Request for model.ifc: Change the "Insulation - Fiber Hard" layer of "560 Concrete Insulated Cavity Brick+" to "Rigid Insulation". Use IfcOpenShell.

First a look at what the model holds.

```python
import ifcopenshell
import ifcopenshell.util.element

model = ifcopenshell.open("model.ifc")
print(model.schema)
for layer_set in model.by_type("IfcMaterialLayerSet"):
    if layer_set.LayerSetName == "560 Concrete Insulated Cavity Brick+":
        for layer in layer_set.MaterialLayers:
            print(layer.id(), layer.Material and layer.Material.Name, layer.LayerThickness, sep=" | ")
        print(len(ifcopenshell.util.element.get_elements_by_material(model, layer_set)), "elements and types use it")
print(sorted(m.Name for m in model.by_type("IfcMaterial") if m.Name)[:60])
```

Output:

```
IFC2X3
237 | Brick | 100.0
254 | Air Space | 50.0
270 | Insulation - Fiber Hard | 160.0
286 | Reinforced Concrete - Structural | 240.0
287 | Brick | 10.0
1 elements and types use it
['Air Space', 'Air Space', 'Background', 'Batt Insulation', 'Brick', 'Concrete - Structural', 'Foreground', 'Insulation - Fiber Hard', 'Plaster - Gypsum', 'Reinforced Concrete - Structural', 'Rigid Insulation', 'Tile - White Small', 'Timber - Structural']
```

```python
import ifcopenshell
import ifcopenshell.api.material

model = ifcopenshell.open("model.ifc")

layer_set = next(s for s in model.by_type("IfcMaterialLayerSet") if s.LayerSetName == "560 Concrete Insulated Cavity Brick+")
layer = next(l for l in layer_set.MaterialLayers if l.Material and l.Material.Name == "Insulation - Fiber Hard")
material = next(m for m in model.by_type("IfcMaterial") if m.Name == "Rigid Insulation")

# Point this one layer at the other material; renaming the old one would change it everywhere.
ifcopenshell.api.material.edit_layer(model, layer=layer, attributes={}, material=material)

print([l.Material.Name if l.Material else None for l in layer_set.MaterialLayers])

model.write("model_edited.ifc")
```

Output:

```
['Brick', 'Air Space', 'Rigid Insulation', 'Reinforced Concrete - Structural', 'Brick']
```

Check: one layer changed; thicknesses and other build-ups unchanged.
